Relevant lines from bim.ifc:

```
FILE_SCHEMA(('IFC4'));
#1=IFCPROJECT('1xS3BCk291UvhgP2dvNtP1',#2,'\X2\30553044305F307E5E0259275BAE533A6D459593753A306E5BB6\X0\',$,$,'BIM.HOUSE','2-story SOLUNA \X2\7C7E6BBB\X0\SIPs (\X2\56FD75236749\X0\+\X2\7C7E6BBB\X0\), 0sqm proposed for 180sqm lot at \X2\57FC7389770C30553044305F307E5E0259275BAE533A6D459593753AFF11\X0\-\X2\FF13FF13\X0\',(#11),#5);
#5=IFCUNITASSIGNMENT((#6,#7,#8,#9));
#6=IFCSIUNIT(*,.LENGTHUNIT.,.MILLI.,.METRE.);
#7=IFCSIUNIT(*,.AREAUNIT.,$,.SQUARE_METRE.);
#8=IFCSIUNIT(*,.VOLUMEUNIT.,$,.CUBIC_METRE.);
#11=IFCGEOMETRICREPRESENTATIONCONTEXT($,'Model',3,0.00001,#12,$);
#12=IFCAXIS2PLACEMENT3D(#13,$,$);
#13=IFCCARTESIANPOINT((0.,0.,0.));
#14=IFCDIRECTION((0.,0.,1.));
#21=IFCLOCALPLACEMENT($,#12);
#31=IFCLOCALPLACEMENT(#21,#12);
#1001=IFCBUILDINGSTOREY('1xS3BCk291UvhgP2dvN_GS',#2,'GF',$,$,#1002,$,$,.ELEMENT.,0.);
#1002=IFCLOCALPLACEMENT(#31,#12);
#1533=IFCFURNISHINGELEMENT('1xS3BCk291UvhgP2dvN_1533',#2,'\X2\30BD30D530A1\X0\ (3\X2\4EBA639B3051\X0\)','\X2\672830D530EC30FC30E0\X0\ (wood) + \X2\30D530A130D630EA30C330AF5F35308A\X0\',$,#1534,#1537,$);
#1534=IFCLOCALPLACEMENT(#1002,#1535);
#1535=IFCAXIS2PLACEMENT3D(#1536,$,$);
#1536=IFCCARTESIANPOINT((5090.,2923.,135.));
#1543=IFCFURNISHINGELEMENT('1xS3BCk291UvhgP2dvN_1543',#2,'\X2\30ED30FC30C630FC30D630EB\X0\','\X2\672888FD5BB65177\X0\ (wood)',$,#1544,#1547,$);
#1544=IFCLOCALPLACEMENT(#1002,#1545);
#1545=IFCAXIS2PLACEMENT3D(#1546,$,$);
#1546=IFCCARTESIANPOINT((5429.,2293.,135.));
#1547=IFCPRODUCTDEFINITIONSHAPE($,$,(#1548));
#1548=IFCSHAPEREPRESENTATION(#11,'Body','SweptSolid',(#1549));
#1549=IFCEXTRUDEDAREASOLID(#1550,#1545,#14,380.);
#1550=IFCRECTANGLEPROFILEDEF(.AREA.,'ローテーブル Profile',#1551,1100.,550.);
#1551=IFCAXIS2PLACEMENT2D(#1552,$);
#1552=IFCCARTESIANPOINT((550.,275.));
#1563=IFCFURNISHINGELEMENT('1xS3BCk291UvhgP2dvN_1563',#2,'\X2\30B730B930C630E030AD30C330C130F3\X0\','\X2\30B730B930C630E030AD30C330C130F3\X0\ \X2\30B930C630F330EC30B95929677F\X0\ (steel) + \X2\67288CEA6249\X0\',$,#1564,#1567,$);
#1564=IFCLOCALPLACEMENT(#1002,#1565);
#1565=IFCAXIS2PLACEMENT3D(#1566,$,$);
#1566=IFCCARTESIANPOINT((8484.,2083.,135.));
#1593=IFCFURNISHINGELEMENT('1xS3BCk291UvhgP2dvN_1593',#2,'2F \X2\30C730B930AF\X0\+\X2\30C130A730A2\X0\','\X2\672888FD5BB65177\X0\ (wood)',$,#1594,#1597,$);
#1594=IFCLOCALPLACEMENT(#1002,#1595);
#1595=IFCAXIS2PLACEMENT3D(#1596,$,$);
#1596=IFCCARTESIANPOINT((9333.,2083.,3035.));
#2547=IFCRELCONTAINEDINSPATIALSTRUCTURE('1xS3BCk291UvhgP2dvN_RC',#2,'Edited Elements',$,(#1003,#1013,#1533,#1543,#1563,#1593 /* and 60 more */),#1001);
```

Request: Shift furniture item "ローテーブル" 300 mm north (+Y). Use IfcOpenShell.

```python
import ifcopenshell
import ifcopenshell.api.geometry
import ifcopenshell.util.placement
import ifcopenshell.util.unit

model = ifcopenshell.open("bim.ifc")
unit_scale = ifcopenshell.util.unit.calculate_unit_scale(model)

item = model.by_guid("1xS3BCk291UvhgP2dvN_1543")
matrix = ifcopenshell.util.placement.get_local_placement(item.ObjectPlacement)
matrix[1, 3] += 0.3 / unit_scale
ifcopenshell.api.geometry.edit_object_placement(model, product=item, matrix=matrix, is_si=False)

print(ifcopenshell.util.placement.get_local_placement(item.ObjectPlacement).round(3) + 0.0)

model.write("bim_edited.ifc")
```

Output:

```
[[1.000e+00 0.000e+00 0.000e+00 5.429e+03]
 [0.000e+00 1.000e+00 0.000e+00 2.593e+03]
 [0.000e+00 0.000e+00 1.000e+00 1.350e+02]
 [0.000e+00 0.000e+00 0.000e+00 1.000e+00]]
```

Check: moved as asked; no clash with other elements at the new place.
